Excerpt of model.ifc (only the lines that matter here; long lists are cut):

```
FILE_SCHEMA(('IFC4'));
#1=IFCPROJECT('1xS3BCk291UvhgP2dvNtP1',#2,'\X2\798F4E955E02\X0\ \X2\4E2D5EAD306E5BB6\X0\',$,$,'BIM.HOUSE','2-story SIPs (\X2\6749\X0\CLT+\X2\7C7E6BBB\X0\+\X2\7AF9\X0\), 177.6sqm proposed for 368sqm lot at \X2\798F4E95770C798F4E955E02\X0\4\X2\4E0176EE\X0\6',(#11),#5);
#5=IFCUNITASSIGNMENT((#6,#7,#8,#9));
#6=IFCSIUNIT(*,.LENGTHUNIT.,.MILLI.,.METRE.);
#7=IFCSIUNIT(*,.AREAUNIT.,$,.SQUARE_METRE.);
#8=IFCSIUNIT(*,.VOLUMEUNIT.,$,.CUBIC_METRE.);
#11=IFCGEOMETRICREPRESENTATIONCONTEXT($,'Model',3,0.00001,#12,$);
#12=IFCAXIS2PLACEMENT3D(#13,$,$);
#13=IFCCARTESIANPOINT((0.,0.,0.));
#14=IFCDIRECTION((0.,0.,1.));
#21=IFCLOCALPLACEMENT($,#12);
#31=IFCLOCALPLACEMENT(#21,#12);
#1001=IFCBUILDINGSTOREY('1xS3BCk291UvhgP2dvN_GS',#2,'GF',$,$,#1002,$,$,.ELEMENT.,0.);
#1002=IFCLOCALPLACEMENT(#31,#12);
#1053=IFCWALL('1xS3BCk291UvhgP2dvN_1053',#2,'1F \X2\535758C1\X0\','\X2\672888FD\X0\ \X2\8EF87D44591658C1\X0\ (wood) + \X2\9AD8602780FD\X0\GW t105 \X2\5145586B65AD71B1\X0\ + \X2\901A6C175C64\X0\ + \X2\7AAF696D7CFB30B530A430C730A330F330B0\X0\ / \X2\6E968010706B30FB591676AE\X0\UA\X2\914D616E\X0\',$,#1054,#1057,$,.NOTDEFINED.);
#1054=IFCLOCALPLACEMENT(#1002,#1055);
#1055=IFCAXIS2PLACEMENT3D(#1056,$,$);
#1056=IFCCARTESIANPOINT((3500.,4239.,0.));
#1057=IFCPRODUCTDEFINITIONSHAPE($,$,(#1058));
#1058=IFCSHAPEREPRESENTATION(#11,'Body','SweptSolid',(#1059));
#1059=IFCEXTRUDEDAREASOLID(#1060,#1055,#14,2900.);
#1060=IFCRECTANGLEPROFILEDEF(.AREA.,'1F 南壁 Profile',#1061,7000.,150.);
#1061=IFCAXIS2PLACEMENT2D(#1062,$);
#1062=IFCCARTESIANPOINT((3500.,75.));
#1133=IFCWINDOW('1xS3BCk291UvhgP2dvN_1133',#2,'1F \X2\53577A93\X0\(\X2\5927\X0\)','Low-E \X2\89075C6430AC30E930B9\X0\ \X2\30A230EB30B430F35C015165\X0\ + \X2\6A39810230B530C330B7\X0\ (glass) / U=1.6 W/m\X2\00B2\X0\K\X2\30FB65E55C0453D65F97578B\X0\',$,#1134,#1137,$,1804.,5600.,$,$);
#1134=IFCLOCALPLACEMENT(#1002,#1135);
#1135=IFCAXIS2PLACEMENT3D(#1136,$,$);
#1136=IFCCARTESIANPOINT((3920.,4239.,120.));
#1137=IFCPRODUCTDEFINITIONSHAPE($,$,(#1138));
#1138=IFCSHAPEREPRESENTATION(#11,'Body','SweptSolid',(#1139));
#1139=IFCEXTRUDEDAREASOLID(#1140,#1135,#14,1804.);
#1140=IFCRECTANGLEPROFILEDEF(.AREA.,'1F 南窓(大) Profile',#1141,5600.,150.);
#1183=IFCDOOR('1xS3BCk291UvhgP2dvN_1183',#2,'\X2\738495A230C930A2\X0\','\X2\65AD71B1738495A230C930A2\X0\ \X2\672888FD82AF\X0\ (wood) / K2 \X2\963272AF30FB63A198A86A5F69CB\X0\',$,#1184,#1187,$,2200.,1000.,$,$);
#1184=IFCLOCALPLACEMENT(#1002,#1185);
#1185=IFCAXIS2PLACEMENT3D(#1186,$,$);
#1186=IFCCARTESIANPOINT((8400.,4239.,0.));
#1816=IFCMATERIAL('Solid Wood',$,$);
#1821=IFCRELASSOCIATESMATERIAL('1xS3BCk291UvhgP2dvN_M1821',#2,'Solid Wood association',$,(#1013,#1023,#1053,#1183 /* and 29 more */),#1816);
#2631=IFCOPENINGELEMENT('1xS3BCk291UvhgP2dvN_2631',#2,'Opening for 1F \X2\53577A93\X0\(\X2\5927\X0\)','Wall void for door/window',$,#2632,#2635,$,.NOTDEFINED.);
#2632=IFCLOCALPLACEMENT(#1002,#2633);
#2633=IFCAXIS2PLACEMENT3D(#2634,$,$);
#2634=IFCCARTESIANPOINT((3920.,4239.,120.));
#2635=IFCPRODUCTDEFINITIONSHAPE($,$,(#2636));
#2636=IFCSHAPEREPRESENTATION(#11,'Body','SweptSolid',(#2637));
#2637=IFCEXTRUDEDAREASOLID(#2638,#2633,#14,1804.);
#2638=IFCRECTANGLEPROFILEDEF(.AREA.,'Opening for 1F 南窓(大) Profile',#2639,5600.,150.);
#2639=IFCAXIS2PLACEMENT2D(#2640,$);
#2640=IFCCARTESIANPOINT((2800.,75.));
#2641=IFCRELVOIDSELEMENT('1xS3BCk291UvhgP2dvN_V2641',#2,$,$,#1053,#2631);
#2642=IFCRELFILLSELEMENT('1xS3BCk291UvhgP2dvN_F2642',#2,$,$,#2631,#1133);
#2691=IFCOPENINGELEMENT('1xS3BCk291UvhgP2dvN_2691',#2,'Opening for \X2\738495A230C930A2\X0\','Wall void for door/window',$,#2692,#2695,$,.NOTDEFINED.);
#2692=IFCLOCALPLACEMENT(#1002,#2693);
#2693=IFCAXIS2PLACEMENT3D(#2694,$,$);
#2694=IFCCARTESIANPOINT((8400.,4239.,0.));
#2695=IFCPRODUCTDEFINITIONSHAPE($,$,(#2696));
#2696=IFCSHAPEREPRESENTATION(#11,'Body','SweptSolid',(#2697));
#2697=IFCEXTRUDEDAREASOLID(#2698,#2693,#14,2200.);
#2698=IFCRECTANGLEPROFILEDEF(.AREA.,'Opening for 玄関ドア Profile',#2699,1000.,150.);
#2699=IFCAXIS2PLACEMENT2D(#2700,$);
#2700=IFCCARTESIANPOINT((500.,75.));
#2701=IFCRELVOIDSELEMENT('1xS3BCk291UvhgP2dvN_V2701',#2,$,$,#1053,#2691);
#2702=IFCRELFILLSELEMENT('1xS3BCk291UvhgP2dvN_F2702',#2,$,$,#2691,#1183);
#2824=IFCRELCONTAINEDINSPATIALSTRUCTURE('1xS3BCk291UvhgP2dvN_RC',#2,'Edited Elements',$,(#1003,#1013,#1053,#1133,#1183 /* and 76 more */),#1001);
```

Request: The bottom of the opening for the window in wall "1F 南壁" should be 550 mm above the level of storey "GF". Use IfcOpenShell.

```python
import numpy as np
import ifcopenshell
import ifcopenshell.api.geometry
import ifcopenshell.geom
import ifcopenshell.util.element
import ifcopenshell.util.placement
import ifcopenshell.util.shape
import ifcopenshell.util.unit

model = ifcopenshell.open("model.ifc")
unit_scale = ifcopenshell.util.unit.calculate_unit_scale(model)

window = model.by_guid("1xS3BCk291UvhgP2dvN_1133")
opening = window.FillsVoids[0].RelatingOpeningElement
storey = ifcopenshell.util.element.get_container(window, ifc_class="IfcBuildingStorey")
level = ifcopenshell.util.placement.get_local_placement(storey.ObjectPlacement)[2, 3]

# The opening's origin need not be at the sill, so measure its lowest point.
shape = ifcopenshell.geom.create_shape(ifcopenshell.geom.settings(), opening)
bottom = ifcopenshell.util.shape.get_shape_bottom_elevation(shape, shape.geometry) / unit_scale
dz = level + 0.55 / unit_scale - bottom

shift = np.array([0.0, 0.0, dz])
# The window is not placed relative to its opening, so move both.
for product in (opening, window):
    matrix = ifcopenshell.util.placement.get_local_placement(product.ObjectPlacement)
    matrix[:3, 3] += shift
    ifcopenshell.api.geometry.edit_object_placement(model, product=product, matrix=matrix, is_si=False)

print(f"moved by {dz * unit_scale:+.3f} m")

model.write("model_updated.ifc")
```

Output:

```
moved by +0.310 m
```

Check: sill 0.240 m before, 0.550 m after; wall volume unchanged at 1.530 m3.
